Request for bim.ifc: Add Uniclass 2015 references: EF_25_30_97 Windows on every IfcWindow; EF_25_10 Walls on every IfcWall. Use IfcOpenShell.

First a look at what the model holds.

```python
import ifcopenshell

model = ifcopenshell.open("bim.ifc")
print(model.schema)
print("classifications:", [c.Name for c in model.by_type("IfcClassification")])
for ifc_class in ("IfcDoor", "IfcRoof", "IfcStair", "IfcWall", "IfcWindow"):
    print(ifc_class, len(model.by_type(ifc_class)))
```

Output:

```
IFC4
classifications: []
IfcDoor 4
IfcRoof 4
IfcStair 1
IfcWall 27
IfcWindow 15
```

```python
import ifcopenshell
import ifcopenshell.api.classification

model = ifcopenshell.open("bim.ifc")

system = ifcopenshell.api.classification.add_classification(model, classification="Uniclass 2015")

codes = {
    "IfcWindow": ("EF_25_30_97", "Windows"),
    "IfcWall": ("EF_25_10", "Walls"),
}
for ifc_class, (code, name) in codes.items():
    products = model.by_type(ifc_class)
    ifcopenshell.api.classification.add_reference(
        model, products=products, classification=system, identification=code, name=name
    )
    print(code, len(products))

model.write("bim-out.ifc")
```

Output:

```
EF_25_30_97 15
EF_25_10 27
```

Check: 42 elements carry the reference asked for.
